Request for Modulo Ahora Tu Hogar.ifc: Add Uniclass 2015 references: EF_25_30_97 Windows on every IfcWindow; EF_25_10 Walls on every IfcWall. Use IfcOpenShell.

First a look at what the model holds.

```python
import ifcopenshell

model = ifcopenshell.open("Modulo Ahora Tu Hogar.ifc")
print(model.schema)
print("classifications:", [c.Name for c in model.by_type("IfcClassification")])
for ifc_class in ("IfcDoor", "IfcRoof", "IfcStair", "IfcWall", "IfcWindow"):
    print(ifc_class, len(model.by_type(ifc_class)))
```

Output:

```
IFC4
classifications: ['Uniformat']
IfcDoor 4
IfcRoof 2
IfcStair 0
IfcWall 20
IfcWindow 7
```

```python
import ifcopenshell
import ifcopenshell.api.classification

model = ifcopenshell.open("Modulo Ahora Tu Hogar.ifc")

system = ifcopenshell.api.classification.add_classification(model, classification="Uniclass 2015")

codes = {
    "IfcWindow": ("EF_25_30_97", "Windows"),
    "IfcWall": ("EF_25_10", "Walls"),
}
for ifc_class, (code, name) in codes.items():
    products = model.by_type(ifc_class)
    ifcopenshell.api.classification.add_reference(
        model, products=products, classification=system, identification=code, name=name
    )
    print(code, len(products))

model.write("Modulo Ahora Tu Hogar_updated.ifc")
```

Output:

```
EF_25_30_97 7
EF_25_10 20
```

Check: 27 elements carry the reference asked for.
